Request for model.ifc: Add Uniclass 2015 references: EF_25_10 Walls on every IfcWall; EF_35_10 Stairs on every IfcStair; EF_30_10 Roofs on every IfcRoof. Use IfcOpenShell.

First a look at what the model holds.

```python
import ifcopenshell

model = ifcopenshell.open("model.ifc")
print(model.schema)
print("classifications:", [c.Name for c in model.by_type("IfcClassification")])
for ifc_class in ("IfcDoor", "IfcRoof", "IfcStair", "IfcWall", "IfcWindow"):
    print(ifc_class, len(model.by_type(ifc_class)))
```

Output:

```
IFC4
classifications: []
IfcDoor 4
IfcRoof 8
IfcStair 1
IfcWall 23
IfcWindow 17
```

```python
import ifcopenshell
import ifcopenshell.api.classification

model = ifcopenshell.open("model.ifc")

system = ifcopenshell.api.classification.add_classification(model, classification="Uniclass 2015")

codes = {
    "IfcWall": ("EF_25_10", "Walls"),
    "IfcStair": ("EF_35_10", "Stairs"),
    "IfcRoof": ("EF_30_10", "Roofs"),
}
for ifc_class, (code, name) in codes.items():
    products = model.by_type(ifc_class)
    ifcopenshell.api.classification.add_reference(
        model, products=products, classification=system, identification=code, name=name
    )
    print(code, len(products))

model.write("model_updated.ifc")
```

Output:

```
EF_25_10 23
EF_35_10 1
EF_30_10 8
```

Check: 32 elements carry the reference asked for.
